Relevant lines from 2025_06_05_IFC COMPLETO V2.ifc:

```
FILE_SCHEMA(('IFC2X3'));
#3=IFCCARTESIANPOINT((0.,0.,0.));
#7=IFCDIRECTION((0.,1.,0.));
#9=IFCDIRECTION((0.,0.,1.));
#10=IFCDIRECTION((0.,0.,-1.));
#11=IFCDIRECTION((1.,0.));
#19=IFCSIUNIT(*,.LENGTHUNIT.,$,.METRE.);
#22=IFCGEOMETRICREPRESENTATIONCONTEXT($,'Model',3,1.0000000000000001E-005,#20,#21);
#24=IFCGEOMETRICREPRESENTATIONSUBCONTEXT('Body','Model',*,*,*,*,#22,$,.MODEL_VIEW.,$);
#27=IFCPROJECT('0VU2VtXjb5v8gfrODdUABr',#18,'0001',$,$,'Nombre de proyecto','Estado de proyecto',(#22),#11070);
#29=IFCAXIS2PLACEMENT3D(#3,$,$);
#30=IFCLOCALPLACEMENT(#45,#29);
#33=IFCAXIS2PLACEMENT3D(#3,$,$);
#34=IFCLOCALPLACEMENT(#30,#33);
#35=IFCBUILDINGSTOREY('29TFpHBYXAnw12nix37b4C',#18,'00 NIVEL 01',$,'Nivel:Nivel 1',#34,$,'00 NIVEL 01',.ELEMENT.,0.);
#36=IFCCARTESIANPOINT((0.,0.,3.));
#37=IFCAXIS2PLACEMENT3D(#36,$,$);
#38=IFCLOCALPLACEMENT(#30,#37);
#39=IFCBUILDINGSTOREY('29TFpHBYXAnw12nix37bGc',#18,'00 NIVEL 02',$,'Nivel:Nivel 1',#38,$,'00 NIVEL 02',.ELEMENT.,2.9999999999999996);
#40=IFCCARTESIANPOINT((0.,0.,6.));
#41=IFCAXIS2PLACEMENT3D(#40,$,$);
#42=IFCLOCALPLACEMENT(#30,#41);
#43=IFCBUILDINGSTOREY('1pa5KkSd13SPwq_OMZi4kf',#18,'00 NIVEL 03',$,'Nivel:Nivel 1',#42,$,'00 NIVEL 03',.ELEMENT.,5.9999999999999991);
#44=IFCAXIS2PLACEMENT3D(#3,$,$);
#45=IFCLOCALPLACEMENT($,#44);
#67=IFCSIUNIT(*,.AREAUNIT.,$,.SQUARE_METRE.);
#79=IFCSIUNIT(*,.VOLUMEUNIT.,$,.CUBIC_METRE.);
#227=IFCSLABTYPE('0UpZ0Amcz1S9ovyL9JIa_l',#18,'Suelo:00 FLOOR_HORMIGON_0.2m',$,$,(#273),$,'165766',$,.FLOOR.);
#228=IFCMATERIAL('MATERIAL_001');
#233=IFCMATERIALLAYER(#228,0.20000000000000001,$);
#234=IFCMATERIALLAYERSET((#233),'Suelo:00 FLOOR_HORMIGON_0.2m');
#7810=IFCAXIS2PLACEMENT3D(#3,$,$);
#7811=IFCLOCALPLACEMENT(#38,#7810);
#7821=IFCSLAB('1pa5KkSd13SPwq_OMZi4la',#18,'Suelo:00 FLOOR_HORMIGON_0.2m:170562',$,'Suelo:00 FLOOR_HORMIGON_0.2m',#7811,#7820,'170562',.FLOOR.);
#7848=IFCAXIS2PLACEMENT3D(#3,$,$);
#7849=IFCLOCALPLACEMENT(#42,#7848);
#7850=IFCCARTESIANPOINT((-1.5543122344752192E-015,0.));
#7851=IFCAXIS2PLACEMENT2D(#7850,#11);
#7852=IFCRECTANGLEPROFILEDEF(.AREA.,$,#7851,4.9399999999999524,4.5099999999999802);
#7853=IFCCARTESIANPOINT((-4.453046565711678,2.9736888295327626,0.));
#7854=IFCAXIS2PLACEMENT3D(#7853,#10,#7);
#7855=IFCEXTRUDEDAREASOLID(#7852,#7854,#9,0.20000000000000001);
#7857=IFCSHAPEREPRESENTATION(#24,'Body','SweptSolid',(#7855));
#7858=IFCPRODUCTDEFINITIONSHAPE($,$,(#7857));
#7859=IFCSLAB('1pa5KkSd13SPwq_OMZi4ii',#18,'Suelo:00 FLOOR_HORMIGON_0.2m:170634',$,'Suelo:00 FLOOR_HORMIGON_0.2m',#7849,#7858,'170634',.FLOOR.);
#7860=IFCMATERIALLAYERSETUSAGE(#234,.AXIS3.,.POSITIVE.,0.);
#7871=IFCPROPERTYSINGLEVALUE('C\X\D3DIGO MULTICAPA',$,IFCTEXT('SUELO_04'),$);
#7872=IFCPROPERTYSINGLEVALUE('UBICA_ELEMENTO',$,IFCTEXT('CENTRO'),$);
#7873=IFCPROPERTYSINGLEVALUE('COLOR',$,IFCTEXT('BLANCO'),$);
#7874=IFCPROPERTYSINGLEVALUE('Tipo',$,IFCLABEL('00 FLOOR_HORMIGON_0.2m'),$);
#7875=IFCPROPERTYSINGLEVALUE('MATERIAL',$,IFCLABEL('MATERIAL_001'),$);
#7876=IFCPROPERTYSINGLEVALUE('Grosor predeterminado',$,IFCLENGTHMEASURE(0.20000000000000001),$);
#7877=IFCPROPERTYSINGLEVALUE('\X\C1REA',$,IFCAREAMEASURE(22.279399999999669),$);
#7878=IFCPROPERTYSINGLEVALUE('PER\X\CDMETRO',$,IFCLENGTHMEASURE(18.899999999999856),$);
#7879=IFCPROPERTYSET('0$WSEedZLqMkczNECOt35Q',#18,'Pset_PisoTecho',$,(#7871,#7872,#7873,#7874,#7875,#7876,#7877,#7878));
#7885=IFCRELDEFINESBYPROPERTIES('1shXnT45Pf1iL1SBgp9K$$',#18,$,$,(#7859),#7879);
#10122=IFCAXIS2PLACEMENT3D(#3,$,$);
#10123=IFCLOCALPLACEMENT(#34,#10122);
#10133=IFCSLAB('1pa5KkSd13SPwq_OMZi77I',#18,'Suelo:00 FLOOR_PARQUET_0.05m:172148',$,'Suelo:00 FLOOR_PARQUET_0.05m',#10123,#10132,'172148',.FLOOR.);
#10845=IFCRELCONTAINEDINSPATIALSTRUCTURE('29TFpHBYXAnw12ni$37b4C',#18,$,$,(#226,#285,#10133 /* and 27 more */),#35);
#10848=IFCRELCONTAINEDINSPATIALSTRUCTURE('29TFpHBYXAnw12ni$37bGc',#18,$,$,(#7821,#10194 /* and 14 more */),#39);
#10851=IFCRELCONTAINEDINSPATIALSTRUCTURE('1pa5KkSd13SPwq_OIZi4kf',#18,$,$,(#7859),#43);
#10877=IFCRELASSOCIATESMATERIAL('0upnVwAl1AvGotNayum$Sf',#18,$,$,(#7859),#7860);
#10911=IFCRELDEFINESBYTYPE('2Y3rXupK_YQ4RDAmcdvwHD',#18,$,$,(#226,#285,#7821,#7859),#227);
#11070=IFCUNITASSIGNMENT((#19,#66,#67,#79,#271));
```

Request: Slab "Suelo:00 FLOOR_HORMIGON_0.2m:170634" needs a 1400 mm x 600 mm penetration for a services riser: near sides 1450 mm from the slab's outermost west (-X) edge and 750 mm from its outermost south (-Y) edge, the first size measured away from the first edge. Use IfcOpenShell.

```python
import numpy as np
import ifcopenshell
import ifcopenshell.api.feature
import ifcopenshell.api.geometry
import ifcopenshell.api.pset
import ifcopenshell.api.root
import ifcopenshell.geom
import ifcopenshell.util.element
import ifcopenshell.util.placement
import ifcopenshell.util.representation
import ifcopenshell.util.shape
import ifcopenshell.util.unit

model = ifcopenshell.open("2025_06_05_IFC COMPLETO V2.ifc")
unit_scale = ifcopenshell.util.unit.calculate_unit_scale(model)
area_scale = ifcopenshell.util.unit.calculate_unit_scale(model, "AREAUNIT")
settings = ifcopenshell.geom.settings()


def volume(element):
    """Net volume in cubic metres, openings subtracted."""
    shape = ifcopenshell.geom.create_shape(settings, element)
    return ifcopenshell.util.shape.get_volume(shape.geometry)


slab = model.by_guid("1pa5KkSd13SPwq_OMZi4ii")
before = volume(slab)

# Extent in the slab's own axes, in metres. The edges named are its -X and -Y sides.
slab_shape = ifcopenshell.geom.create_shape(settings, slab)
vertices = ifcopenshell.util.shape.get_vertices(slab_shape.geometry)
x_min, y_min, bottom = vertices.min(axis=0)
top = vertices[:, 2].max()

opening = ifcopenshell.api.root.create_entity(model, ifc_class="IfcOpeningElement", name="Services riser opening")
context = ifcopenshell.util.representation.get_context(model, "Model", "Body", "MODEL_VIEW")
width, depth = 1.4, 0.6
outline = [(0.0, 0.0), (width, 0.0), (width, depth), (0.0, depth), (0.0, 0.0)]
# Overshoot both faces by 50 mm so the cut is clean.
shape = ifcopenshell.api.geometry.add_slab_representation(
    model, context=context, depth=top - bottom + 0.1, polyline=outline
)
ifcopenshell.api.geometry.assign_representation(model, product=opening, representation=shape)

matrix = ifcopenshell.util.placement.get_local_placement(slab.ObjectPlacement)
matrix[:, 3] = matrix @ np.append(np.array([x_min + 1.45, y_min + 0.75, bottom - 0.05]) / unit_scale, 1.0)
ifcopenshell.api.geometry.edit_object_placement(model, product=opening, matrix=matrix, is_si=False)
ifcopenshell.api.feature.add_feature(model, feature=opening, element=slab)

after = volume(slab)

# Update the slab's stored quantities.
pset = model.by_id(ifcopenshell.util.element.get_pset(slab, "Pset_PisoTecho", should_inherit=False)["id"])
ifcopenshell.api.pset.edit_pset(model, pset=pset, properties={
    "ÁREA": model.create_entity("IfcAreaMeasure", after / (top - bottom) / area_scale),
})

print(f"slab volume {before:.3f} -> {after:.3f} m3")

model.write("2025_06_05_IFC COMPLETO V2-out.ifc")
```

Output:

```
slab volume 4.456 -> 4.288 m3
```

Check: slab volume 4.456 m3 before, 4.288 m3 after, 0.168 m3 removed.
